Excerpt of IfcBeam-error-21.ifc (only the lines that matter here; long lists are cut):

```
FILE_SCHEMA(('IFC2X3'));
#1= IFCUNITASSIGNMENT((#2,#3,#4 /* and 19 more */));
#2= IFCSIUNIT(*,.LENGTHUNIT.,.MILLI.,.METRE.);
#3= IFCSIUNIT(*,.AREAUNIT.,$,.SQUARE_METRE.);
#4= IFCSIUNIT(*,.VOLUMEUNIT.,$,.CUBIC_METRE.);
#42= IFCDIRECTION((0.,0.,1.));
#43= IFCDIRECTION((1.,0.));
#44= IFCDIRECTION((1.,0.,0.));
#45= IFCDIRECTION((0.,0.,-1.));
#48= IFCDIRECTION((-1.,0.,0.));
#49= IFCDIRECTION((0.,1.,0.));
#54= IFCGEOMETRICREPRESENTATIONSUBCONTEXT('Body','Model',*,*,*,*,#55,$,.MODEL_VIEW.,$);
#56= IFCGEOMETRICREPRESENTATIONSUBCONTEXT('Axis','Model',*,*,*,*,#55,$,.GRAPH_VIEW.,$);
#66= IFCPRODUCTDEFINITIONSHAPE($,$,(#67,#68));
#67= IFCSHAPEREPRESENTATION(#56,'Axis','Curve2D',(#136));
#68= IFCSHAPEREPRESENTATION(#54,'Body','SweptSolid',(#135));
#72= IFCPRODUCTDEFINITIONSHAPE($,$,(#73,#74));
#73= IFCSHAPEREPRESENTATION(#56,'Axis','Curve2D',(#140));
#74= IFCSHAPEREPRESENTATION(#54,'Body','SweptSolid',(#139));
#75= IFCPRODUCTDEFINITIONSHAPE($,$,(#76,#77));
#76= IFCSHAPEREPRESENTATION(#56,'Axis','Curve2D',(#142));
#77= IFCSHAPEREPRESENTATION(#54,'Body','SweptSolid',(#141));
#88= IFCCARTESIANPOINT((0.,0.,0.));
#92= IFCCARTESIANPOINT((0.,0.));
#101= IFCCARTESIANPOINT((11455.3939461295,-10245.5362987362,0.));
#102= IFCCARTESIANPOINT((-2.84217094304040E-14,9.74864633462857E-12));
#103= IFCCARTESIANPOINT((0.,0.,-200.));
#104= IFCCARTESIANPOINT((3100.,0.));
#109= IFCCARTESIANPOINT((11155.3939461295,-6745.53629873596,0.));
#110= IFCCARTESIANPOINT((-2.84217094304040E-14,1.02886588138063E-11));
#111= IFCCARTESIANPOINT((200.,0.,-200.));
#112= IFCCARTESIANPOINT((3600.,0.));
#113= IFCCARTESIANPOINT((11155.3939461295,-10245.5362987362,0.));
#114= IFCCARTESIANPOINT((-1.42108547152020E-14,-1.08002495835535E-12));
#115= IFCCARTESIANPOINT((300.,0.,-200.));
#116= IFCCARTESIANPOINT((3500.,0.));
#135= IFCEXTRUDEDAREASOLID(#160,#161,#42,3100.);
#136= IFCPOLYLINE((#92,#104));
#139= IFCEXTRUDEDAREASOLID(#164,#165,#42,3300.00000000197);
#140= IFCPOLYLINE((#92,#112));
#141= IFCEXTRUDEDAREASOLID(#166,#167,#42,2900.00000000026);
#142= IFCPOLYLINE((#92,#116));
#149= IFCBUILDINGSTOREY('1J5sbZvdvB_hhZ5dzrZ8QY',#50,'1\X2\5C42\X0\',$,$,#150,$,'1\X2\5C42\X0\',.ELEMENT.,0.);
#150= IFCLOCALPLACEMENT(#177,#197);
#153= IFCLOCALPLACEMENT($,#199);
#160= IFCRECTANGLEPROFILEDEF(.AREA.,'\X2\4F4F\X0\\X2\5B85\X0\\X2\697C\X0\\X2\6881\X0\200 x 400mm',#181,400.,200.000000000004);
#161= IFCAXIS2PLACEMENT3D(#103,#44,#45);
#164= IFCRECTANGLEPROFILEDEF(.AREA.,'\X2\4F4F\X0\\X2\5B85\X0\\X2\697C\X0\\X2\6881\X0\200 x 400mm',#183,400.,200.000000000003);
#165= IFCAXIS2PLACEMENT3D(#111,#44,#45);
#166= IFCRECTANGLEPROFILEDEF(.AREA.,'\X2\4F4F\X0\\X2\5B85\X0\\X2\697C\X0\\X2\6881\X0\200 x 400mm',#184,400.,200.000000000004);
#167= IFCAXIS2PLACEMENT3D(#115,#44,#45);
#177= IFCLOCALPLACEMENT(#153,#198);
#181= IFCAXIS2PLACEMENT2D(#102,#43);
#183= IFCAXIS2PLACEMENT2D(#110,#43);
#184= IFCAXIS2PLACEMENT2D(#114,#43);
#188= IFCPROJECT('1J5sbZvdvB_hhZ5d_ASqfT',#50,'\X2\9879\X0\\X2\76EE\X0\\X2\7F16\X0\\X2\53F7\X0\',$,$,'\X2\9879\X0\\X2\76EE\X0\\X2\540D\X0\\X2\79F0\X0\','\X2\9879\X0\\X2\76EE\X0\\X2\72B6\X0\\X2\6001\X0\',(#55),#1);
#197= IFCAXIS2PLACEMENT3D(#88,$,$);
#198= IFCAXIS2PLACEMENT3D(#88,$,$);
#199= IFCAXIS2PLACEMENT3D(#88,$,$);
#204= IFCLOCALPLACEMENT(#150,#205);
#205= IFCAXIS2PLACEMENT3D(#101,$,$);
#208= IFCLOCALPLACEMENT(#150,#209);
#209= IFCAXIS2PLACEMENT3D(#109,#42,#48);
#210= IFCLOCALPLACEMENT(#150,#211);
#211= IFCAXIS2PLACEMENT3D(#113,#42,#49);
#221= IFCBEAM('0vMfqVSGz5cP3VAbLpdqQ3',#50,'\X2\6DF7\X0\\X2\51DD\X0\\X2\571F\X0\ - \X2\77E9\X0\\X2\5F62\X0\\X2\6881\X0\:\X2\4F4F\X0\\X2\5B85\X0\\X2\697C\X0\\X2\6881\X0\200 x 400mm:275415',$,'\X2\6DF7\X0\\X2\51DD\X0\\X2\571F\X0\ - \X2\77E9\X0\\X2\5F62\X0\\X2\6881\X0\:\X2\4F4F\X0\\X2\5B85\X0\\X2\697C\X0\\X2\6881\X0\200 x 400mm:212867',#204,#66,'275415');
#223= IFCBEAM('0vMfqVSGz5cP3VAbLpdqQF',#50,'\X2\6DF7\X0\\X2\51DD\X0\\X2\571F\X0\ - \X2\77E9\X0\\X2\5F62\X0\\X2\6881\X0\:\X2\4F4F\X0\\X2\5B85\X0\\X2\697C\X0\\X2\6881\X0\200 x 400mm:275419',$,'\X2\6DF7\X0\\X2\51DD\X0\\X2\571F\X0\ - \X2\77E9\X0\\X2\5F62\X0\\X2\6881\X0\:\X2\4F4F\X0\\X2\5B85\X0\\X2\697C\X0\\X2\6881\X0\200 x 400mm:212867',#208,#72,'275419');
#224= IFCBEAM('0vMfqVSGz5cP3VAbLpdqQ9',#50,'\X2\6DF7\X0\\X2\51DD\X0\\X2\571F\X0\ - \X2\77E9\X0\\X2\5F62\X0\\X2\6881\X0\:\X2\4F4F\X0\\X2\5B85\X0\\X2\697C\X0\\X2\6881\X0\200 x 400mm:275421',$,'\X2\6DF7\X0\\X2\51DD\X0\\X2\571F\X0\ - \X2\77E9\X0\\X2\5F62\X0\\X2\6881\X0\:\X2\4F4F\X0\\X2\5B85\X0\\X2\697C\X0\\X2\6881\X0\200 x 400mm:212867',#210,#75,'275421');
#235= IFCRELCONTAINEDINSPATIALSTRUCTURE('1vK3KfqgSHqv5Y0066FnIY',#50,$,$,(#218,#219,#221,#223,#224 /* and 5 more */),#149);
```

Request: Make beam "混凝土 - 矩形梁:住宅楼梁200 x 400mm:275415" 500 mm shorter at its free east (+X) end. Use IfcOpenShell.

```python
import numpy as np
import ifcopenshell
import ifcopenshell.util.representation
import ifcopenshell.util.unit

model = ifcopenshell.open("IfcBeam-error-21.ifc")
unit_scale = ifcopenshell.util.unit.calculate_unit_scale(model)

member = model.by_guid("0vMfqVSGz5cP3VAbLpdqQ3")
change = -0.5 / unit_scale

# The extrusion runs towards the end named, so only its depth changes.
body = ifcopenshell.util.representation.get_representation(member, "Model", "Body")
solid = body.Items[0]
old_length = solid.Depth
solid.Depth += change

# Move the axis end point with it.
axis = next(r for r in member.Representation.Representations if r.RepresentationIdentifier == "Axis").Items[0]
start, end = (np.array(p.Coordinates) for p in axis.Points)
end = end + (end - start) / np.linalg.norm(end - start) * change
point = model.createIfcCartesianPoint(end.tolist())
axis.Points = [axis.Points[0], point]

print(f"length {old_length:g} -> {solid.Depth:g}")

model.write("IfcBeam-error-21_v2.ifc")
```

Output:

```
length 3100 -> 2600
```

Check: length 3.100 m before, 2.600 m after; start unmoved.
